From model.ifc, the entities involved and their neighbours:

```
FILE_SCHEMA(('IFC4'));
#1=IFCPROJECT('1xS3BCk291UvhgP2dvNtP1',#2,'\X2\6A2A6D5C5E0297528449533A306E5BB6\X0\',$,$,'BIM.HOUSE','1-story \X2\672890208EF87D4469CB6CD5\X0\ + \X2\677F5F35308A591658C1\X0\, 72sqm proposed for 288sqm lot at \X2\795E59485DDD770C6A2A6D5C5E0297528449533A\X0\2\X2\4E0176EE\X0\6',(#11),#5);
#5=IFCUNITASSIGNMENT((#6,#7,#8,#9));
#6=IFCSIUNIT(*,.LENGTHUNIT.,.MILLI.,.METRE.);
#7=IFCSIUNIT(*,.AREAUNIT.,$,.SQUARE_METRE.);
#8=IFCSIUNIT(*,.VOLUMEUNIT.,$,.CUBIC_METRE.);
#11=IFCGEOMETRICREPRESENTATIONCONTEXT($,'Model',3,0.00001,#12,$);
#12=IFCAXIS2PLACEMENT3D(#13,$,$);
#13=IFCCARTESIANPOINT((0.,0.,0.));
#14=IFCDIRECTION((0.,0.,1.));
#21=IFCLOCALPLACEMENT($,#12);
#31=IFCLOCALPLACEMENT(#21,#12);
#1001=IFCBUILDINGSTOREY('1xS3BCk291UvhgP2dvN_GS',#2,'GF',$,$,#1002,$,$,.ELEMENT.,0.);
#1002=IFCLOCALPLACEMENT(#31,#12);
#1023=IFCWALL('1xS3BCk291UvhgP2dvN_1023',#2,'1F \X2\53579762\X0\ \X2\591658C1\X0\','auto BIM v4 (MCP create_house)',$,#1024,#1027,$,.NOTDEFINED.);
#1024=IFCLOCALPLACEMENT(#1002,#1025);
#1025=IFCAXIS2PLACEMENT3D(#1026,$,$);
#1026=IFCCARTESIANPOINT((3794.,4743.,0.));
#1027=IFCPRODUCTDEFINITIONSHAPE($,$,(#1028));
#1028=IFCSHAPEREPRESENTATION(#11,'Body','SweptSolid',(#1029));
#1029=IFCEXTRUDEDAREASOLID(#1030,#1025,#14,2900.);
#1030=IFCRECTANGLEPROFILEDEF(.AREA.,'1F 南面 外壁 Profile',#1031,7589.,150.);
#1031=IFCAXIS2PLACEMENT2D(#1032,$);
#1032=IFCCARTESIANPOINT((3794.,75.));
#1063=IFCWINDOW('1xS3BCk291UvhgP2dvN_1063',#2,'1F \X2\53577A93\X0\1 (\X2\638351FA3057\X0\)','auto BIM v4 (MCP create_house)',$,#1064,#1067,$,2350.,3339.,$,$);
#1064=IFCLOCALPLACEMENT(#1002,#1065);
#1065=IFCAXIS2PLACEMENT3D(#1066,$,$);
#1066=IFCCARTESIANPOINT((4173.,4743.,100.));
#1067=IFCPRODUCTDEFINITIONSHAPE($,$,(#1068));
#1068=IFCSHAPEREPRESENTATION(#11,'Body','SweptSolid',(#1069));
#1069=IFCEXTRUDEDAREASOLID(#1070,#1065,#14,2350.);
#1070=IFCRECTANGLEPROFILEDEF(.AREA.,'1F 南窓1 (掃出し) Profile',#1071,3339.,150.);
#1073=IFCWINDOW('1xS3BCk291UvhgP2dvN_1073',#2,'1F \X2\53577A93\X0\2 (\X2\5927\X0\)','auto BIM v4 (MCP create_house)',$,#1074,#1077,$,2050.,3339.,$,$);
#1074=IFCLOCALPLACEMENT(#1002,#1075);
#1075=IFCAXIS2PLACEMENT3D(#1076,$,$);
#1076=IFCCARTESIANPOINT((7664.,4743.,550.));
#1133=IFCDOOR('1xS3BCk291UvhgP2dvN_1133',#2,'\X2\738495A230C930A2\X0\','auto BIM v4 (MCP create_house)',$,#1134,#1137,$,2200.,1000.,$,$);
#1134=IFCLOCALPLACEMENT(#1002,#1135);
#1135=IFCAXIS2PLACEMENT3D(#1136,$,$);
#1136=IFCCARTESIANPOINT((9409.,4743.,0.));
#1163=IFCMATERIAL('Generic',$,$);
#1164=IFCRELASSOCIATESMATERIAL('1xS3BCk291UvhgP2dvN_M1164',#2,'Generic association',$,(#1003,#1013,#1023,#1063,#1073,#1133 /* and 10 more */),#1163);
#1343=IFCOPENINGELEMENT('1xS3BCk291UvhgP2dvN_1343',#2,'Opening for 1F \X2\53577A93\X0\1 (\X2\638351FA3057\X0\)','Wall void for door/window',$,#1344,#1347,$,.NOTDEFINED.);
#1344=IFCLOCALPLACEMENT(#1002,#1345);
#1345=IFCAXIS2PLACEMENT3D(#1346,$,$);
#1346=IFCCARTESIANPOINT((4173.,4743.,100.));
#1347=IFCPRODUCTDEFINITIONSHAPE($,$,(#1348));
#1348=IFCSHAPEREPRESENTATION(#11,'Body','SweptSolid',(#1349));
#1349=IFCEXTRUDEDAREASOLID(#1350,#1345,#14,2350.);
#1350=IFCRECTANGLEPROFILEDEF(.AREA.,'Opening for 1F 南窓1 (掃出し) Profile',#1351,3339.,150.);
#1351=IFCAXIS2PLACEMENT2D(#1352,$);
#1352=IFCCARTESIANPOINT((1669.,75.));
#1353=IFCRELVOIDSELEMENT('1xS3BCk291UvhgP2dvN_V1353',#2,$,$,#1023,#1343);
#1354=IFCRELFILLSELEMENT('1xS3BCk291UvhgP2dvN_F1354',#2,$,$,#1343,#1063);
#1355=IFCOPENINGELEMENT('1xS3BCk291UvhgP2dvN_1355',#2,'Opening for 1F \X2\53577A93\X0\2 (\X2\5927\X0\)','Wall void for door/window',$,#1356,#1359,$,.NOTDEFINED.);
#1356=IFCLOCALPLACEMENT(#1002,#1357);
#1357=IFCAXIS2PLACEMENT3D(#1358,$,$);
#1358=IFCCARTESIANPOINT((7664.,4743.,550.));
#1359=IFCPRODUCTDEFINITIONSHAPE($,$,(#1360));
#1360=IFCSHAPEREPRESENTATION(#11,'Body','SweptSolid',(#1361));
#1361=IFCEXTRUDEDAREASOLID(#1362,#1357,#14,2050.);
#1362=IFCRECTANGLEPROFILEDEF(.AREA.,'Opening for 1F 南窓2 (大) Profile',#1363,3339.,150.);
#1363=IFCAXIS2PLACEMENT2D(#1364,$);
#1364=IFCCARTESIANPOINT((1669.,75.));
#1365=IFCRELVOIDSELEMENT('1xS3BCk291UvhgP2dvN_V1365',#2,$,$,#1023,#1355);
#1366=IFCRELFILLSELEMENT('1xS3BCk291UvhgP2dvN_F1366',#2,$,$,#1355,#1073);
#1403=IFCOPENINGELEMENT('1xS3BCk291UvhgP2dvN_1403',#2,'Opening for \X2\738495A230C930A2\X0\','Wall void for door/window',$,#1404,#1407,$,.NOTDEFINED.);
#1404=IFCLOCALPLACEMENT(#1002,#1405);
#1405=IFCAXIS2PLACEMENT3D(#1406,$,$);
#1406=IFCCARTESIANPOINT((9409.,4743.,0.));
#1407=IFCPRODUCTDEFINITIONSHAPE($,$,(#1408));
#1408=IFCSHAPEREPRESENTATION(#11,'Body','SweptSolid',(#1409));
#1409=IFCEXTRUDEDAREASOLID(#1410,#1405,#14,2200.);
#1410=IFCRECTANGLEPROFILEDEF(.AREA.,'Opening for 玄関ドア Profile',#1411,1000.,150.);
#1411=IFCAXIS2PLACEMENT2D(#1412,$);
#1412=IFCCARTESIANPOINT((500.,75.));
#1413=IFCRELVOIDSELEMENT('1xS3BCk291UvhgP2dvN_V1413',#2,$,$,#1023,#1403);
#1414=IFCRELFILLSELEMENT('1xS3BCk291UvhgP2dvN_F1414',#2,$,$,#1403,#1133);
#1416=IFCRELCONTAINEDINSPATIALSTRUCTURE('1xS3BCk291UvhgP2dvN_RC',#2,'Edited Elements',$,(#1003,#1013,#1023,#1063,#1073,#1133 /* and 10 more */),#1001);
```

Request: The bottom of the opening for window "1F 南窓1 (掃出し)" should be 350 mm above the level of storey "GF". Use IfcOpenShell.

```python
import numpy as np
import ifcopenshell
import ifcopenshell.api.geometry
import ifcopenshell.geom
import ifcopenshell.util.element
import ifcopenshell.util.placement
import ifcopenshell.util.shape
import ifcopenshell.util.unit

model = ifcopenshell.open("model.ifc")
unit_scale = ifcopenshell.util.unit.calculate_unit_scale(model)

window = model.by_guid("1xS3BCk291UvhgP2dvN_1063")
opening = window.FillsVoids[0].RelatingOpeningElement
storey = ifcopenshell.util.element.get_container(window, ifc_class="IfcBuildingStorey")
level = ifcopenshell.util.placement.get_local_placement(storey.ObjectPlacement)[2, 3]

# The opening's origin need not be at the sill, so measure its lowest point.
shape = ifcopenshell.geom.create_shape(ifcopenshell.geom.settings(), opening)
bottom = ifcopenshell.util.shape.get_shape_bottom_elevation(shape, shape.geometry) / unit_scale
dz = level + 0.35 / unit_scale - bottom

shift = np.array([0.0, 0.0, dz])
# The window is not placed relative to its opening, so move both.
for product in (opening, window):
    matrix = ifcopenshell.util.placement.get_local_placement(product.ObjectPlacement)
    matrix[:3, 3] += shift
    ifcopenshell.api.geometry.edit_object_placement(model, product=product, matrix=matrix, is_si=False)

print(f"moved by {dz * unit_scale:+.3f} m")

model.write("model-out.ifc")
```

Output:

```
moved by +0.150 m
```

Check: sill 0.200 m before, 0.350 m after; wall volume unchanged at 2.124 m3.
